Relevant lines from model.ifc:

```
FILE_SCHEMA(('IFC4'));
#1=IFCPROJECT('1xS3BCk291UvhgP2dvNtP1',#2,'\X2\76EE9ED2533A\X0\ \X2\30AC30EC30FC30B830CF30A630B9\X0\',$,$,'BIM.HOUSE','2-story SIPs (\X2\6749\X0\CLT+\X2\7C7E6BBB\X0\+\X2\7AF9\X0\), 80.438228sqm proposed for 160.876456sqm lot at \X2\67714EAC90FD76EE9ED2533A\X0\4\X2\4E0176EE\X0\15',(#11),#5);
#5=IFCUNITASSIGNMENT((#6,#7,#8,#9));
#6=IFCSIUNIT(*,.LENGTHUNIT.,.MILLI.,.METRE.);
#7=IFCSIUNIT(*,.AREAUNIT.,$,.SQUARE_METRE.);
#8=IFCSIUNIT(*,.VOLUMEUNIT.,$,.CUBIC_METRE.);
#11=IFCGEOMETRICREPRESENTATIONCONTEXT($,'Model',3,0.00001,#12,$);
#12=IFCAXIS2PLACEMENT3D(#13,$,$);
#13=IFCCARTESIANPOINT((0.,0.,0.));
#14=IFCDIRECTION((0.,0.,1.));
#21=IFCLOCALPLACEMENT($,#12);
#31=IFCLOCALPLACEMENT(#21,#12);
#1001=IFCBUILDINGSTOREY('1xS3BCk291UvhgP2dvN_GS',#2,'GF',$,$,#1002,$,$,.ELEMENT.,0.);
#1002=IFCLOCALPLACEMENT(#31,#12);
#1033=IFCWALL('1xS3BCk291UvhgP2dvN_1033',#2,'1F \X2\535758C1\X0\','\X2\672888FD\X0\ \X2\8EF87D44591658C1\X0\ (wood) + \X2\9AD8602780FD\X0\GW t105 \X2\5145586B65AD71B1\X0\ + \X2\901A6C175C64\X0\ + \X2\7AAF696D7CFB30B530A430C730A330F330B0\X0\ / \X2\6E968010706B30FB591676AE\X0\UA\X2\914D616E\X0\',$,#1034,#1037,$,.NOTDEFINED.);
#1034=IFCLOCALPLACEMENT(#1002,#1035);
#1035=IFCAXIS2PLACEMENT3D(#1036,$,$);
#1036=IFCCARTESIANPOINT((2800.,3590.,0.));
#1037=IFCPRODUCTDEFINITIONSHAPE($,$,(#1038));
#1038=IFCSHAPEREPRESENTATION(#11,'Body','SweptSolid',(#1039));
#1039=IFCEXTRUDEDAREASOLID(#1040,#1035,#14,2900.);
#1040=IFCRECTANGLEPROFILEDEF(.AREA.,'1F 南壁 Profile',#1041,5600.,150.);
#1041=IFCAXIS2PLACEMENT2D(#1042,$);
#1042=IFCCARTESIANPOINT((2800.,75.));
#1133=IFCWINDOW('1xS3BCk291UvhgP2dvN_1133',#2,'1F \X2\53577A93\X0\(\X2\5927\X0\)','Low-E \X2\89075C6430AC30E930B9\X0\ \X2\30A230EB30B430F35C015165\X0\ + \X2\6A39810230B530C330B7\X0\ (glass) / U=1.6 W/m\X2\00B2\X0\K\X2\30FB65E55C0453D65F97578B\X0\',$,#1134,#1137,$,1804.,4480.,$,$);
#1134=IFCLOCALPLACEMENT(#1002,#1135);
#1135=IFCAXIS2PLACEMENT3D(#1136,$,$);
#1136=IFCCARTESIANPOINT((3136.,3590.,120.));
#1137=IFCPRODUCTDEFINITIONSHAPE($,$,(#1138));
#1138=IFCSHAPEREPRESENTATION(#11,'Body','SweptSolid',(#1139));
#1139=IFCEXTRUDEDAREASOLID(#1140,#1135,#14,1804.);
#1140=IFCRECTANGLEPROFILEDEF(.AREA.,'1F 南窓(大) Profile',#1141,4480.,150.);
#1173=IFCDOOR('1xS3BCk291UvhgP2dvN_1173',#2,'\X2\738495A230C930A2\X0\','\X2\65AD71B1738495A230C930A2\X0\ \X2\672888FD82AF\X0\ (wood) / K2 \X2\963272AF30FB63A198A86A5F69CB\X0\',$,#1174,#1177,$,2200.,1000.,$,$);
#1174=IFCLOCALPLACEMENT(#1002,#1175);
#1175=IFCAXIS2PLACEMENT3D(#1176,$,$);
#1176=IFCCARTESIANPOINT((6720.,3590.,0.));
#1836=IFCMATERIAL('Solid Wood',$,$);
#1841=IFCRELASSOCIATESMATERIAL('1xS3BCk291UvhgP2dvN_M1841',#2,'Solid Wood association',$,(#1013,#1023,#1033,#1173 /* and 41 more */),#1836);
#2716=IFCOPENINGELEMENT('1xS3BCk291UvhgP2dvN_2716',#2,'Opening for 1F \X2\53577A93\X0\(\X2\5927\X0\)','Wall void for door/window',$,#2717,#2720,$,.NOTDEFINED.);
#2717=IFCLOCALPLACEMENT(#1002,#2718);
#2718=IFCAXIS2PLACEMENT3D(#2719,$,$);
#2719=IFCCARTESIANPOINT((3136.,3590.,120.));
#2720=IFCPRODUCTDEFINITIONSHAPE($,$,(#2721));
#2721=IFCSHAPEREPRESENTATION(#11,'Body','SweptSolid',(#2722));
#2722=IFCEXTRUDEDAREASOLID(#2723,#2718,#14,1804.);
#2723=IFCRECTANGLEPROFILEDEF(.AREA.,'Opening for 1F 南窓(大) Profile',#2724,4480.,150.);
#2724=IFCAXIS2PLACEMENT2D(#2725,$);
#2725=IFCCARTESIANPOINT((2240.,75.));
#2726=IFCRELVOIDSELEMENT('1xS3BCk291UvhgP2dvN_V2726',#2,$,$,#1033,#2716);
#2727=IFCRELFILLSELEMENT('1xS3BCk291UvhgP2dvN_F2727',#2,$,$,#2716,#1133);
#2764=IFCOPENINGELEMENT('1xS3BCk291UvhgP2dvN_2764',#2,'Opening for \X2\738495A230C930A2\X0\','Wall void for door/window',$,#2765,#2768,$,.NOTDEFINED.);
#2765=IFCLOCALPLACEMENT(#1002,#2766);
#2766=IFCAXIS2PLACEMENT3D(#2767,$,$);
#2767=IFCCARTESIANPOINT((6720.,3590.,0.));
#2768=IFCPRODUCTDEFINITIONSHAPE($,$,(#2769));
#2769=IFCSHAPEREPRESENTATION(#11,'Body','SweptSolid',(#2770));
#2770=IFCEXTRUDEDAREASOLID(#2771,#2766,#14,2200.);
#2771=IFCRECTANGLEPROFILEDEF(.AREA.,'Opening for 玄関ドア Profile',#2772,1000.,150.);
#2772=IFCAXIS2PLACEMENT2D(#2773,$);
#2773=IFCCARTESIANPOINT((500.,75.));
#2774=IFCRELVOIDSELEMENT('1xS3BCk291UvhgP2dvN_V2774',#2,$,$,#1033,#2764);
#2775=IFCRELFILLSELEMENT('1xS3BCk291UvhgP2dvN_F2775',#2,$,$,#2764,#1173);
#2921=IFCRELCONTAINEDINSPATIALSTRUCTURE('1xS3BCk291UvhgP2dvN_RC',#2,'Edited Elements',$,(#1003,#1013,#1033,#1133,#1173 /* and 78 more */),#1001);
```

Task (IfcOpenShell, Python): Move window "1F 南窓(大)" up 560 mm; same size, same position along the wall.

```python
import numpy as np
import ifcopenshell
import ifcopenshell.api.geometry
import ifcopenshell.util.placement
import ifcopenshell.util.unit

model = ifcopenshell.open("model.ifc")
unit_scale = ifcopenshell.util.unit.calculate_unit_scale(model)

window = model.by_guid("1xS3BCk291UvhgP2dvN_1133")
opening = window.FillsVoids[0].RelatingOpeningElement
dz = 0.56 / unit_scale

shift = np.array([0.0, 0.0, dz])
# The window is not placed relative to its opening, so move both.
for product in (opening, window):
    matrix = ifcopenshell.util.placement.get_local_placement(product.ObjectPlacement)
    matrix[:3, 3] += shift
    ifcopenshell.api.geometry.edit_object_placement(model, product=product, matrix=matrix, is_si=False)

print(f"moved by {dz * unit_scale:+.3f} m")

model.write("model_v2.ifc")
```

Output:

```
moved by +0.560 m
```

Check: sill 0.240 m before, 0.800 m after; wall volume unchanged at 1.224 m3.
